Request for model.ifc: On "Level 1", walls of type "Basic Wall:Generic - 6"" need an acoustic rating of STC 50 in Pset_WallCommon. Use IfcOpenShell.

First a look at what the model holds.

```python
import ifcopenshell
import ifcopenshell.util.element

model = ifcopenshell.open("model.ifc")
print(model.schema)
storey = next(s for s in model.by_type("IfcBuildingStorey") if s.Name == "Level 1")
walls = [e for e in ifcopenshell.util.element.get_decomposition(storey) if e.is_a("IfcWall")]
seen = {}
for e in walls:
    element_type = ifcopenshell.util.element.get_type(e)
    key = (element_type.Name if element_type != e and element_type else None, ifcopenshell.util.element.get_pset(e, "Pset_WallCommon", "AcousticRating"))
    seen[key] = seen.get(key, 0) + 1
for (name, value), count in sorted(seen.items(), key=str):
    print(count, "x", name, "|", value)
```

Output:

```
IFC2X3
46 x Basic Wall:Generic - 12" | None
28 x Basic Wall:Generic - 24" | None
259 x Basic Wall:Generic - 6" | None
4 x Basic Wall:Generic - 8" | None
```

```python
import ifcopenshell
import ifcopenshell.api.pset
import ifcopenshell.util.element

model = ifcopenshell.open("model.ifc")

storey = next(s for s in model.by_type("IfcBuildingStorey") if s.Name == "Level 1")
walls = [e for e in ifcopenshell.util.element.get_decomposition(storey) if e.is_a("IfcWall")]

count = 0
for e in walls:
    element_type = ifcopenshell.util.element.get_type(e)
    if element_type in (None, e) or element_type.Name != 'Basic Wall:Generic - 6"':
        continue
    # add_pset returns the element's existing set when there is one.
    pset = ifcopenshell.api.pset.add_pset(model, product=e, name="Pset_WallCommon")
    ifcopenshell.api.pset.edit_pset(model, pset=pset, properties={"AcousticRating": "STC 50"})
    count += 1

print(count, "walls updated")

model.write("model_updated.ifc")
```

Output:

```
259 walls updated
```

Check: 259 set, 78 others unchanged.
